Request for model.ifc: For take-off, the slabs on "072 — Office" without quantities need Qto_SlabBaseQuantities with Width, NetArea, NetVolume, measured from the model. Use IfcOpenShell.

First a look at what the model holds.

```python
import ifcopenshell
import ifcopenshell.util.element
import ifcopenshell.util.unit

model = ifcopenshell.open("model.ifc")
print(model.schema)
for unit_type in ("LENGTHUNIT", "AREAUNIT", "VOLUMEUNIT"):
    print(unit_type, ifcopenshell.util.unit.calculate_unit_scale(model, unit_type))
storey = next(s for s in model.by_type("IfcBuildingStorey") if s.Name == "072 — Office")
slabs = [e for e in ifcopenshell.util.element.get_decomposition(storey) if e.is_a("IfcSlab")]
for e in sorted(slabs, key=lambda e: e.id()):
    print(e.id(), e.is_a(), e.Name, list(ifcopenshell.util.element.get_psets(e, qtos_only=True)), sep=" | ")
```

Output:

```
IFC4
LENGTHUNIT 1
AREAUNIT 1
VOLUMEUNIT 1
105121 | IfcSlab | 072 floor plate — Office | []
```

```python
import ifcopenshell
import ifcopenshell.api.pset
import ifcopenshell.geom
import ifcopenshell.util.element
import ifcopenshell.util.shape
import ifcopenshell.util.unit

model = ifcopenshell.open("model.ifc")
unit_scale = ifcopenshell.util.unit.calculate_unit_scale(model)
area_scale = ifcopenshell.util.unit.calculate_unit_scale(model, "AREAUNIT")
volume_scale = ifcopenshell.util.unit.calculate_unit_scale(model, "VOLUMEUNIT")
settings = ifcopenshell.geom.settings()

storey = next(s for s in model.by_type("IfcBuildingStorey") if s.Name == "072 — Office")
slabs = [e for e in ifcopenshell.util.element.get_decomposition(storey) if e.is_a("IfcSlab")]

for e in sorted(slabs, key=lambda e: e.id()):
    if ifcopenshell.util.element.get_psets(e, qtos_only=True, should_inherit=False):
        continue
    # Geometry comes back in metres, in the element's own axes.
    shape = ifcopenshell.geom.create_shape(settings, e)
    values = {
        "Width": ifcopenshell.util.shape.get_z(shape.geometry) / unit_scale,
        "NetArea": ifcopenshell.util.shape.get_footprint_area(shape.geometry) / area_scale,
        "NetVolume": ifcopenshell.util.shape.get_volume(shape.geometry) / volume_scale,
    }
    qto = ifcopenshell.api.pset.add_qto(model, product=e, name="Qto_SlabBaseQuantities")
    ifcopenshell.api.pset.edit_qto(model, qto=qto, properties=values)
    print(e.id(), {k: round(v, 3) for k, v in values.items()})

model.write("model-out.ifc")
```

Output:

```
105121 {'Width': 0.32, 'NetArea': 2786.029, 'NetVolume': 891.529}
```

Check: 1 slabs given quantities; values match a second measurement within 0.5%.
